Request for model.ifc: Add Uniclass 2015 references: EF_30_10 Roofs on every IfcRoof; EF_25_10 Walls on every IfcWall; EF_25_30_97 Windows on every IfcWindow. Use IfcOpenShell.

First a look at what the model holds.

```python
import ifcopenshell

model = ifcopenshell.open("model.ifc")
print(model.schema)
print("classifications:", [c.Name for c in model.by_type("IfcClassification")])
for ifc_class in ("IfcDoor", "IfcRoof", "IfcStair", "IfcWall", "IfcWindow"):
    print(ifc_class, len(model.by_type(ifc_class)))
```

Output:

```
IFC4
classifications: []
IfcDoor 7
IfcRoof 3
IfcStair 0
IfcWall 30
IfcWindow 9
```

```python
import ifcopenshell
import ifcopenshell.api.classification

model = ifcopenshell.open("model.ifc")

system = ifcopenshell.api.classification.add_classification(model, classification="Uniclass 2015")

codes = {
    "IfcRoof": ("EF_30_10", "Roofs"),
    "IfcWall": ("EF_25_10", "Walls"),
    "IfcWindow": ("EF_25_30_97", "Windows"),
}
for ifc_class, (code, name) in codes.items():
    products = model.by_type(ifc_class)
    ifcopenshell.api.classification.add_reference(
        model, products=products, classification=system, identification=code, name=name
    )
    print(code, len(products))

model.write("model_v2.ifc")
```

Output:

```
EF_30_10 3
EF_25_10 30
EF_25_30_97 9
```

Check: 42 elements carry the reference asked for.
